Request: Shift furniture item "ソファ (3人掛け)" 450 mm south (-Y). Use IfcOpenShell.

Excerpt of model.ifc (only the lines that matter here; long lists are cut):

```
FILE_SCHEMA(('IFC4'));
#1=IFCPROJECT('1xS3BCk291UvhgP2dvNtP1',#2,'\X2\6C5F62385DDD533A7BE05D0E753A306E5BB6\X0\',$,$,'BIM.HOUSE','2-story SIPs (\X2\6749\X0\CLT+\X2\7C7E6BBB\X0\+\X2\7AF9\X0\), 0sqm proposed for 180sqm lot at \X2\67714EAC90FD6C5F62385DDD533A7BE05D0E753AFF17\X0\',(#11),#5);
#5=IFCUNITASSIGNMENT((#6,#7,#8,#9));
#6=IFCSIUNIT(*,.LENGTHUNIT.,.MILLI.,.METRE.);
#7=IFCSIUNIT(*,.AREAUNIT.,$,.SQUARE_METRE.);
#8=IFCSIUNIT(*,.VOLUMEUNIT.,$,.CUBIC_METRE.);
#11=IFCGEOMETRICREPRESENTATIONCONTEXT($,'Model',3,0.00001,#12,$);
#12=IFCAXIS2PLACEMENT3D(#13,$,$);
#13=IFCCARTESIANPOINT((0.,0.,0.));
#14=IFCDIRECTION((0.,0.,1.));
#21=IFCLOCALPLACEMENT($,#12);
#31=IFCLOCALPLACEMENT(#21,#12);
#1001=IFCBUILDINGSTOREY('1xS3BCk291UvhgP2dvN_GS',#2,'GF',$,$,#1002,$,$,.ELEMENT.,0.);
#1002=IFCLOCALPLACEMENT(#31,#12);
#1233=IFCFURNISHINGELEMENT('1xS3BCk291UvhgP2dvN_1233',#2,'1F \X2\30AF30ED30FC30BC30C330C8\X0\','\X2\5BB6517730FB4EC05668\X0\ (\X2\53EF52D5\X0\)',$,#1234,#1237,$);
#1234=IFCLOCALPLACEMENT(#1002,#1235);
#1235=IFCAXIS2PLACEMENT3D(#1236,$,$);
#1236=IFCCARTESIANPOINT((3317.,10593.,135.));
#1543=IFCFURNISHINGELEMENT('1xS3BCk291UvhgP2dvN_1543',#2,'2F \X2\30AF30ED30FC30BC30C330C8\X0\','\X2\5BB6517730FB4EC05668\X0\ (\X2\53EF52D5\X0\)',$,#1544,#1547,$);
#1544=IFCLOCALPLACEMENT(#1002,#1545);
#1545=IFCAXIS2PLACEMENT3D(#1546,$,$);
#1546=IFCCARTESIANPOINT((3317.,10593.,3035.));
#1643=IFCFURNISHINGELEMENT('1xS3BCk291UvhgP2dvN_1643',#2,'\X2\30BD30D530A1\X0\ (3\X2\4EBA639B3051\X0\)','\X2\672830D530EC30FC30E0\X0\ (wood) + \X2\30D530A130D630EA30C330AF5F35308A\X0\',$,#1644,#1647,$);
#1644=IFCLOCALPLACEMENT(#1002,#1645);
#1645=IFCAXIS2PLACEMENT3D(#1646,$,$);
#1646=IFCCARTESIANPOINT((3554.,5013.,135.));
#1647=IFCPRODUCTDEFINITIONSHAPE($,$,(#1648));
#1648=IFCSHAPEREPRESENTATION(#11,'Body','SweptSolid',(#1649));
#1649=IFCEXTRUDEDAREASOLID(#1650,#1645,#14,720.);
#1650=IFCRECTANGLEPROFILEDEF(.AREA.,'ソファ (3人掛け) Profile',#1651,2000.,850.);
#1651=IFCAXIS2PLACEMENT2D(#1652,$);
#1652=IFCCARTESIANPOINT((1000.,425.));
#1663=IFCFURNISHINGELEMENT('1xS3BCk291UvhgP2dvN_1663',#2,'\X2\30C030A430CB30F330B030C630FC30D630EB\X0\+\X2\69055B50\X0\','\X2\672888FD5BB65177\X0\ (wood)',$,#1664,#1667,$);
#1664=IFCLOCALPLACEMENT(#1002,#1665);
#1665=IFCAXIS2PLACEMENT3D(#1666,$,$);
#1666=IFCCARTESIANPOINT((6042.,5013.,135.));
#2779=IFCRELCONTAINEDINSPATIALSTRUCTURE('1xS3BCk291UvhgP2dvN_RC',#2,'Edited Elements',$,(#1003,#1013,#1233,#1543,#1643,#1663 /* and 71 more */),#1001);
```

```python
import ifcopenshell
import ifcopenshell.api.geometry
import ifcopenshell.util.placement

model = ifcopenshell.open("model.ifc")

item = model.by_guid("1xS3BCk291UvhgP2dvN_1643")
matrix = ifcopenshell.util.placement.get_local_placement(item.ObjectPlacement)
matrix[1, 3] -= 450.0
ifcopenshell.api.geometry.edit_object_placement(model, product=item, matrix=matrix, is_si=False)

print(ifcopenshell.util.placement.get_local_placement(item.ObjectPlacement).round(3) + 0.0)

model.write("model-out.ifc")
```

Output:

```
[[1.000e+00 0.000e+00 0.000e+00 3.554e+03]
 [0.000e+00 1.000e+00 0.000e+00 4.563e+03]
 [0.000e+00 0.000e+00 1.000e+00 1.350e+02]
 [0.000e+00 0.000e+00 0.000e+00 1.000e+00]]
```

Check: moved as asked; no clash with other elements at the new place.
